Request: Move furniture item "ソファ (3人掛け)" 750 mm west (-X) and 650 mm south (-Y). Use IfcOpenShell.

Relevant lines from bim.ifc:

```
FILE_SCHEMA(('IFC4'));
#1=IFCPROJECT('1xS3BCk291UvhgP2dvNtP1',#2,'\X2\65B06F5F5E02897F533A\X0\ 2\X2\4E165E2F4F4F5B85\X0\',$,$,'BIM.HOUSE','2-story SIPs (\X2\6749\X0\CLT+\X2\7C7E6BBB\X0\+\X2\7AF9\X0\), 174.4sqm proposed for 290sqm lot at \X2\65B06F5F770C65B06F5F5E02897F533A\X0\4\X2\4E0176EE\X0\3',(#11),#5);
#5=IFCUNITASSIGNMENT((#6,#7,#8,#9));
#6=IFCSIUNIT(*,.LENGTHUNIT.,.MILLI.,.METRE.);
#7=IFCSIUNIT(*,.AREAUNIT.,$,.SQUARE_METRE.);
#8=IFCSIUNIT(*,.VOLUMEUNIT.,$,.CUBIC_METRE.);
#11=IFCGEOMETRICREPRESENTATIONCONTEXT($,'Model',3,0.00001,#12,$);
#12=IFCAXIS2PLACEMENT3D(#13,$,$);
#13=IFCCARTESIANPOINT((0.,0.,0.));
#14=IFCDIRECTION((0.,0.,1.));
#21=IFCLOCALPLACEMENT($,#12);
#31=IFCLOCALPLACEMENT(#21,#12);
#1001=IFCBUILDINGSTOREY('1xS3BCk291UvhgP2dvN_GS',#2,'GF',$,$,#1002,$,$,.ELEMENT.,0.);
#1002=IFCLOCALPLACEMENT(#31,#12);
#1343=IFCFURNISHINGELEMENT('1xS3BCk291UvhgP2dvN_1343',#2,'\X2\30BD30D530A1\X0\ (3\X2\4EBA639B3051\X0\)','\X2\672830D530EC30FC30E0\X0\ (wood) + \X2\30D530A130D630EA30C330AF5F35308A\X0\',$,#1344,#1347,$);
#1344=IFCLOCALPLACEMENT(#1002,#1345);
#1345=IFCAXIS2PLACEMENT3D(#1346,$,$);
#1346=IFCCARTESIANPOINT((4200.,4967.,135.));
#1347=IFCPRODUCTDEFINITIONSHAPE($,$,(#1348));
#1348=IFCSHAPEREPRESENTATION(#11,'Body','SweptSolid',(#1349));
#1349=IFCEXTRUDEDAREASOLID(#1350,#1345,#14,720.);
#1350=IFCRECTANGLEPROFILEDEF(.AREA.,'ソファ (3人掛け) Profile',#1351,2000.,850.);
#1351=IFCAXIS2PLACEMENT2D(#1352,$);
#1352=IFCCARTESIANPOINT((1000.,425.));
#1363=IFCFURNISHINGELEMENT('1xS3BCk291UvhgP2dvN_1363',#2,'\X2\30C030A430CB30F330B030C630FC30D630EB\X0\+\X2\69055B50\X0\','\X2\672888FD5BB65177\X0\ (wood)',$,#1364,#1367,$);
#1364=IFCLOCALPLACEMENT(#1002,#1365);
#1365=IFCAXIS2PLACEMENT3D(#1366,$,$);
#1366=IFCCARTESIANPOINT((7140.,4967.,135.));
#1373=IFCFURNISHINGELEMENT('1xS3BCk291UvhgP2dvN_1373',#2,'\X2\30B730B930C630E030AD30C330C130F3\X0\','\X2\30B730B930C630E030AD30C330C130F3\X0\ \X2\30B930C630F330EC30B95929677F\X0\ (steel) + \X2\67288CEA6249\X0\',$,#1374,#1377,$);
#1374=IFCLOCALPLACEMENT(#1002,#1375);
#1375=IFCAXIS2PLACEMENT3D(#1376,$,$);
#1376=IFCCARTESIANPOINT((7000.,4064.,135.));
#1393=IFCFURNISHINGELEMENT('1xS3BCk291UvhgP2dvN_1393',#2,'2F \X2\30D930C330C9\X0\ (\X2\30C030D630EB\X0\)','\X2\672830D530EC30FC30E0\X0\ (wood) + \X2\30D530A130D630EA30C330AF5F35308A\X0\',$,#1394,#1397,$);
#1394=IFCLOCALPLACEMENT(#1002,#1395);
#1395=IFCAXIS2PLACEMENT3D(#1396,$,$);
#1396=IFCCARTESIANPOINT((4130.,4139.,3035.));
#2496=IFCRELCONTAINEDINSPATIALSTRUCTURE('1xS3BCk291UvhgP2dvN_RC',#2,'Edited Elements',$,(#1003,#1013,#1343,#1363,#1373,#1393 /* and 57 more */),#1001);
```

```python
import ifcopenshell
import ifcopenshell.api.geometry
import ifcopenshell.util.placement

model = ifcopenshell.open("bim.ifc")

item = model.by_guid("1xS3BCk291UvhgP2dvN_1343")
matrix = ifcopenshell.util.placement.get_local_placement(item.ObjectPlacement)
matrix[0, 3] -= 750.0
matrix[1, 3] -= 650.0
ifcopenshell.api.geometry.edit_object_placement(model, product=item, matrix=matrix, is_si=False)

print(ifcopenshell.util.placement.get_local_placement(item.ObjectPlacement).round(3) + 0.0)

model.write("bim_v2.ifc")
```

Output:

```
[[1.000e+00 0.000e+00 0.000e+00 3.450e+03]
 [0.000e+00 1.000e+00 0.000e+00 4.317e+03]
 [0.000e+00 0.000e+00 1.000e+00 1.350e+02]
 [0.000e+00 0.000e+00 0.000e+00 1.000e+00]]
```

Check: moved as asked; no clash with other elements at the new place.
